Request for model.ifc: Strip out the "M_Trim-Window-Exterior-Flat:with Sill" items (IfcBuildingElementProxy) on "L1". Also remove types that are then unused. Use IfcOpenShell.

First a look at what the model holds.

```python
import ifcopenshell
import ifcopenshell.util.element

model = ifcopenshell.open("model.ifc")
print(model.schema)
storey = next(s for s in model.by_type("IfcBuildingStorey") if s.Name == "L1")
proxies = [e for e in ifcopenshell.util.element.get_decomposition(storey) if e.is_a("IfcBuildingElementProxy")]
seen = {}
for e in proxies:
    element_type = ifcopenshell.util.element.get_type(e)
    name = element_type.Name if element_type not in (None, e) else None
    seen[name] = seen.get(name, 0) + 1
for name, count in sorted(seen.items(), key=str):
    print(count, "x", name)
```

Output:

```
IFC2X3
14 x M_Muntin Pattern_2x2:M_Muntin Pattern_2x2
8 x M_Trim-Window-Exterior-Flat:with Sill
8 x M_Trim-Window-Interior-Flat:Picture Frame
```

```python
import ifcopenshell
import ifcopenshell.api.root
import ifcopenshell.util.element

model = ifcopenshell.open("model.ifc")

storey = next(s for s in model.by_type("IfcBuildingStorey") if s.Name == "L1")
proxies = [e for e in ifcopenshell.util.element.get_decomposition(storey) if e.is_a("IfcBuildingElementProxy")]
targets = [e for e in proxies if (t := ifcopenshell.util.element.get_type(e)) not in (None, e) and t.Name == "M_Trim-Window-Exterior-Flat:with Sill"]
types = {ifcopenshell.util.element.get_type(e) for e in targets} - {None, *targets}

for e in targets:
    ifcopenshell.api.root.remove_product(model, product=e)
print(len(targets), "removed")

unused = [t for t in types if not ifcopenshell.util.element.get_types(t)]
for t in unused:
    ifcopenshell.api.root.remove_product(model, product=t)
print(len(unused), "unused types removed")

model.write("model-out.ifc")
```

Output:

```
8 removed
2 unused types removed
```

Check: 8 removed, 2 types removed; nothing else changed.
